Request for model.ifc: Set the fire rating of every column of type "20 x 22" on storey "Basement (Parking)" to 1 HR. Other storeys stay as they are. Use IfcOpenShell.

First a look at what the model holds.

```python
import ifcopenshell
import ifcopenshell.util.element

model = ifcopenshell.open("model.ifc")
print(model.schema)
storey = next(s for s in model.by_type("IfcBuildingStorey") if s.Name == "Basement (Parking)")
columns = [e for e in ifcopenshell.util.element.get_decomposition(storey) if e.is_a("IfcColumn")]
seen = {}
for e in columns:
    element_type = ifcopenshell.util.element.get_type(e)
    key = (element_type.Name if element_type != e and element_type else None, ifcopenshell.util.element.get_pset(e, "Pset_ColumnCommon", "FireRating"))
    seen[key] = seen.get(key, 0) + 1
for (name, value), count in sorted(seen.items(), key=str):
    print(count, "x", name, "|", value)
```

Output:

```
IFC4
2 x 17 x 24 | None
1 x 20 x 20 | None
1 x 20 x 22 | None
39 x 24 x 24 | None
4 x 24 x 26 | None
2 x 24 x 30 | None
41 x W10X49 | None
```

```python
import ifcopenshell
import ifcopenshell.api.pset
import ifcopenshell.util.element

model = ifcopenshell.open("model.ifc")

storey = next(s for s in model.by_type("IfcBuildingStorey") if s.Name == "Basement (Parking)")
columns = [e for e in ifcopenshell.util.element.get_decomposition(storey) if e.is_a("IfcColumn")]

count = 0
for e in columns:
    element_type = ifcopenshell.util.element.get_type(e)
    if element_type in (None, e) or element_type.Name != "20 x 22":
        continue
    # add_pset returns the element's existing set when there is one.
    pset = ifcopenshell.api.pset.add_pset(model, product=e, name="Pset_ColumnCommon")
    ifcopenshell.api.pset.edit_pset(model, pset=pset, properties={"FireRating": "1 HR"})
    count += 1

print(count, "columns updated")

model.write("model_v2.ifc")
```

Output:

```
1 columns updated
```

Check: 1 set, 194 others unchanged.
